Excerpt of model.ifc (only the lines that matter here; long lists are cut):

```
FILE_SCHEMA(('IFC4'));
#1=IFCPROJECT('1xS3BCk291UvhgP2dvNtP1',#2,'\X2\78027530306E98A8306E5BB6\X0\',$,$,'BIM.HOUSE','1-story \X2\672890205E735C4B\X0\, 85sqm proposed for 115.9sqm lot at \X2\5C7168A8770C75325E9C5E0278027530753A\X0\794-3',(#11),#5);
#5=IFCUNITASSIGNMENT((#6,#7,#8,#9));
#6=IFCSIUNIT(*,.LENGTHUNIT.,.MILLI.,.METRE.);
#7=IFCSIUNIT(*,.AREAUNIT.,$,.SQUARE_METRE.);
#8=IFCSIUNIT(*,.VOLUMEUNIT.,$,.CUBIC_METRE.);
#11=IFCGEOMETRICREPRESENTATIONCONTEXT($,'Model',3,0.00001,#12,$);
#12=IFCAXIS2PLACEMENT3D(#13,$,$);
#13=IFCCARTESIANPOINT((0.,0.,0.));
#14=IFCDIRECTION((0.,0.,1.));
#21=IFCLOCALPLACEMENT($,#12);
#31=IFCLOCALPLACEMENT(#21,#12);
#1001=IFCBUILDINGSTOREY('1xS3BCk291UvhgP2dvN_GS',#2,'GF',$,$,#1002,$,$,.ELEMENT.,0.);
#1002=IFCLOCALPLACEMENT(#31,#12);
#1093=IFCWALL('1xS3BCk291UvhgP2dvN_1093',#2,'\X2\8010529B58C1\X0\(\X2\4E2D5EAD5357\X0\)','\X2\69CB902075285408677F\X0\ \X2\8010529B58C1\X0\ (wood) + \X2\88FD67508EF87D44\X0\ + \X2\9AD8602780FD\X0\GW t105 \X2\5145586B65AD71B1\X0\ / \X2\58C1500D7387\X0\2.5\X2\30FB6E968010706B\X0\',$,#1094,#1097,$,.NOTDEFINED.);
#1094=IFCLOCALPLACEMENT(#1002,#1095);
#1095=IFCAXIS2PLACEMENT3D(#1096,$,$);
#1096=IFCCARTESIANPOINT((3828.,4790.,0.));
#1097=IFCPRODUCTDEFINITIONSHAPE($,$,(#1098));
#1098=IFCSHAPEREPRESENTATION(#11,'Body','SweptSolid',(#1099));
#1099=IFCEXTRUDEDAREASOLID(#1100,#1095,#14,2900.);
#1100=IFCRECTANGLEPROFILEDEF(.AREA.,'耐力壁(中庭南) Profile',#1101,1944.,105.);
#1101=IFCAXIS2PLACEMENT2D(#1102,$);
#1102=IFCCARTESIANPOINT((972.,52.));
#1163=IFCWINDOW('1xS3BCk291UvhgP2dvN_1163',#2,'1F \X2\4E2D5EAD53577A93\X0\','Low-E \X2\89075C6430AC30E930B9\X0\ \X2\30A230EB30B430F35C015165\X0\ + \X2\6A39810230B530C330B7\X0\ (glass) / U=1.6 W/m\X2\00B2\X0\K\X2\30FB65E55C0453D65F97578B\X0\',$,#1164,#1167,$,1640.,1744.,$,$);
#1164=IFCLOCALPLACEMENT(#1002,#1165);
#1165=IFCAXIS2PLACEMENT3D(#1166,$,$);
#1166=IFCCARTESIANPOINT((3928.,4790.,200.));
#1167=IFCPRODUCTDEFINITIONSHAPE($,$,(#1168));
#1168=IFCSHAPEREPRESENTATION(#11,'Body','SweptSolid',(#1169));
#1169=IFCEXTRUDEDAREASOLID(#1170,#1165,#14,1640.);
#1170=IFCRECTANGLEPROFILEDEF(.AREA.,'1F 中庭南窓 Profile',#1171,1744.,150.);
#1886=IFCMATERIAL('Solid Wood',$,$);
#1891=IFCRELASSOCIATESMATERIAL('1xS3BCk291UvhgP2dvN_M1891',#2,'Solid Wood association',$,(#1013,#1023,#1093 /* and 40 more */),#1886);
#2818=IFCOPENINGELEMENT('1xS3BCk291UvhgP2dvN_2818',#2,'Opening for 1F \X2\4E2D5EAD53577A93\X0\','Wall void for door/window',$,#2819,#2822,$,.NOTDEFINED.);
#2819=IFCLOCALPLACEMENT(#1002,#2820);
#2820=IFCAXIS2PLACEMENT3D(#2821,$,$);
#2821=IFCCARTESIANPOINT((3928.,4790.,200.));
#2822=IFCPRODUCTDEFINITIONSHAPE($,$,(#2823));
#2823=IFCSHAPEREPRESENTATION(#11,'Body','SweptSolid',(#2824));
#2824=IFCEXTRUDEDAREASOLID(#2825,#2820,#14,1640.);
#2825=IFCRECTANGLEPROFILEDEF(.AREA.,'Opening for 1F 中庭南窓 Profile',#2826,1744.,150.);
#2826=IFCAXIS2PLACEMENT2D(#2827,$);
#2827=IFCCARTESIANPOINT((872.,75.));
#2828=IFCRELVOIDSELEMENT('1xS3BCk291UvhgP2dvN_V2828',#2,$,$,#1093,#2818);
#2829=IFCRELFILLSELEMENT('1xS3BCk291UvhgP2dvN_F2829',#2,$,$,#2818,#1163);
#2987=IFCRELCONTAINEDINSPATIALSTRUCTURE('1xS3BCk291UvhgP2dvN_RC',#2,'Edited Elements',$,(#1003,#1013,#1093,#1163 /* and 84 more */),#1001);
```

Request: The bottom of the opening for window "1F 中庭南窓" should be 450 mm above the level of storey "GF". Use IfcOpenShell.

```python
import numpy as np
import ifcopenshell
import ifcopenshell.api.geometry
import ifcopenshell.geom
import ifcopenshell.util.element
import ifcopenshell.util.placement
import ifcopenshell.util.shape
import ifcopenshell.util.unit

model = ifcopenshell.open("model.ifc")
unit_scale = ifcopenshell.util.unit.calculate_unit_scale(model)

window = model.by_guid("1xS3BCk291UvhgP2dvN_1163")
opening = window.FillsVoids[0].RelatingOpeningElement
storey = ifcopenshell.util.element.get_container(window, ifc_class="IfcBuildingStorey")
level = ifcopenshell.util.placement.get_local_placement(storey.ObjectPlacement)[2, 3]

# The opening's origin need not be at the sill, so measure its lowest point.
shape = ifcopenshell.geom.create_shape(ifcopenshell.geom.settings(), opening)
bottom = ifcopenshell.util.shape.get_shape_bottom_elevation(shape, shape.geometry) / unit_scale
dz = level + 0.45 / unit_scale - bottom

shift = np.array([0.0, 0.0, dz])
# The window is not placed relative to its opening, so move both.
for product in (opening, window):
    matrix = ifcopenshell.util.placement.get_local_placement(product.ObjectPlacement)
    matrix[:3, 3] += shift
    ifcopenshell.api.geometry.edit_object_placement(model, product=product, matrix=matrix, is_si=False)

print(f"moved by {dz * unit_scale:+.3f} m")

model.write("model-out.ifc")
```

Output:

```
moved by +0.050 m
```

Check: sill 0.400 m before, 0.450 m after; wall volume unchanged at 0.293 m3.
